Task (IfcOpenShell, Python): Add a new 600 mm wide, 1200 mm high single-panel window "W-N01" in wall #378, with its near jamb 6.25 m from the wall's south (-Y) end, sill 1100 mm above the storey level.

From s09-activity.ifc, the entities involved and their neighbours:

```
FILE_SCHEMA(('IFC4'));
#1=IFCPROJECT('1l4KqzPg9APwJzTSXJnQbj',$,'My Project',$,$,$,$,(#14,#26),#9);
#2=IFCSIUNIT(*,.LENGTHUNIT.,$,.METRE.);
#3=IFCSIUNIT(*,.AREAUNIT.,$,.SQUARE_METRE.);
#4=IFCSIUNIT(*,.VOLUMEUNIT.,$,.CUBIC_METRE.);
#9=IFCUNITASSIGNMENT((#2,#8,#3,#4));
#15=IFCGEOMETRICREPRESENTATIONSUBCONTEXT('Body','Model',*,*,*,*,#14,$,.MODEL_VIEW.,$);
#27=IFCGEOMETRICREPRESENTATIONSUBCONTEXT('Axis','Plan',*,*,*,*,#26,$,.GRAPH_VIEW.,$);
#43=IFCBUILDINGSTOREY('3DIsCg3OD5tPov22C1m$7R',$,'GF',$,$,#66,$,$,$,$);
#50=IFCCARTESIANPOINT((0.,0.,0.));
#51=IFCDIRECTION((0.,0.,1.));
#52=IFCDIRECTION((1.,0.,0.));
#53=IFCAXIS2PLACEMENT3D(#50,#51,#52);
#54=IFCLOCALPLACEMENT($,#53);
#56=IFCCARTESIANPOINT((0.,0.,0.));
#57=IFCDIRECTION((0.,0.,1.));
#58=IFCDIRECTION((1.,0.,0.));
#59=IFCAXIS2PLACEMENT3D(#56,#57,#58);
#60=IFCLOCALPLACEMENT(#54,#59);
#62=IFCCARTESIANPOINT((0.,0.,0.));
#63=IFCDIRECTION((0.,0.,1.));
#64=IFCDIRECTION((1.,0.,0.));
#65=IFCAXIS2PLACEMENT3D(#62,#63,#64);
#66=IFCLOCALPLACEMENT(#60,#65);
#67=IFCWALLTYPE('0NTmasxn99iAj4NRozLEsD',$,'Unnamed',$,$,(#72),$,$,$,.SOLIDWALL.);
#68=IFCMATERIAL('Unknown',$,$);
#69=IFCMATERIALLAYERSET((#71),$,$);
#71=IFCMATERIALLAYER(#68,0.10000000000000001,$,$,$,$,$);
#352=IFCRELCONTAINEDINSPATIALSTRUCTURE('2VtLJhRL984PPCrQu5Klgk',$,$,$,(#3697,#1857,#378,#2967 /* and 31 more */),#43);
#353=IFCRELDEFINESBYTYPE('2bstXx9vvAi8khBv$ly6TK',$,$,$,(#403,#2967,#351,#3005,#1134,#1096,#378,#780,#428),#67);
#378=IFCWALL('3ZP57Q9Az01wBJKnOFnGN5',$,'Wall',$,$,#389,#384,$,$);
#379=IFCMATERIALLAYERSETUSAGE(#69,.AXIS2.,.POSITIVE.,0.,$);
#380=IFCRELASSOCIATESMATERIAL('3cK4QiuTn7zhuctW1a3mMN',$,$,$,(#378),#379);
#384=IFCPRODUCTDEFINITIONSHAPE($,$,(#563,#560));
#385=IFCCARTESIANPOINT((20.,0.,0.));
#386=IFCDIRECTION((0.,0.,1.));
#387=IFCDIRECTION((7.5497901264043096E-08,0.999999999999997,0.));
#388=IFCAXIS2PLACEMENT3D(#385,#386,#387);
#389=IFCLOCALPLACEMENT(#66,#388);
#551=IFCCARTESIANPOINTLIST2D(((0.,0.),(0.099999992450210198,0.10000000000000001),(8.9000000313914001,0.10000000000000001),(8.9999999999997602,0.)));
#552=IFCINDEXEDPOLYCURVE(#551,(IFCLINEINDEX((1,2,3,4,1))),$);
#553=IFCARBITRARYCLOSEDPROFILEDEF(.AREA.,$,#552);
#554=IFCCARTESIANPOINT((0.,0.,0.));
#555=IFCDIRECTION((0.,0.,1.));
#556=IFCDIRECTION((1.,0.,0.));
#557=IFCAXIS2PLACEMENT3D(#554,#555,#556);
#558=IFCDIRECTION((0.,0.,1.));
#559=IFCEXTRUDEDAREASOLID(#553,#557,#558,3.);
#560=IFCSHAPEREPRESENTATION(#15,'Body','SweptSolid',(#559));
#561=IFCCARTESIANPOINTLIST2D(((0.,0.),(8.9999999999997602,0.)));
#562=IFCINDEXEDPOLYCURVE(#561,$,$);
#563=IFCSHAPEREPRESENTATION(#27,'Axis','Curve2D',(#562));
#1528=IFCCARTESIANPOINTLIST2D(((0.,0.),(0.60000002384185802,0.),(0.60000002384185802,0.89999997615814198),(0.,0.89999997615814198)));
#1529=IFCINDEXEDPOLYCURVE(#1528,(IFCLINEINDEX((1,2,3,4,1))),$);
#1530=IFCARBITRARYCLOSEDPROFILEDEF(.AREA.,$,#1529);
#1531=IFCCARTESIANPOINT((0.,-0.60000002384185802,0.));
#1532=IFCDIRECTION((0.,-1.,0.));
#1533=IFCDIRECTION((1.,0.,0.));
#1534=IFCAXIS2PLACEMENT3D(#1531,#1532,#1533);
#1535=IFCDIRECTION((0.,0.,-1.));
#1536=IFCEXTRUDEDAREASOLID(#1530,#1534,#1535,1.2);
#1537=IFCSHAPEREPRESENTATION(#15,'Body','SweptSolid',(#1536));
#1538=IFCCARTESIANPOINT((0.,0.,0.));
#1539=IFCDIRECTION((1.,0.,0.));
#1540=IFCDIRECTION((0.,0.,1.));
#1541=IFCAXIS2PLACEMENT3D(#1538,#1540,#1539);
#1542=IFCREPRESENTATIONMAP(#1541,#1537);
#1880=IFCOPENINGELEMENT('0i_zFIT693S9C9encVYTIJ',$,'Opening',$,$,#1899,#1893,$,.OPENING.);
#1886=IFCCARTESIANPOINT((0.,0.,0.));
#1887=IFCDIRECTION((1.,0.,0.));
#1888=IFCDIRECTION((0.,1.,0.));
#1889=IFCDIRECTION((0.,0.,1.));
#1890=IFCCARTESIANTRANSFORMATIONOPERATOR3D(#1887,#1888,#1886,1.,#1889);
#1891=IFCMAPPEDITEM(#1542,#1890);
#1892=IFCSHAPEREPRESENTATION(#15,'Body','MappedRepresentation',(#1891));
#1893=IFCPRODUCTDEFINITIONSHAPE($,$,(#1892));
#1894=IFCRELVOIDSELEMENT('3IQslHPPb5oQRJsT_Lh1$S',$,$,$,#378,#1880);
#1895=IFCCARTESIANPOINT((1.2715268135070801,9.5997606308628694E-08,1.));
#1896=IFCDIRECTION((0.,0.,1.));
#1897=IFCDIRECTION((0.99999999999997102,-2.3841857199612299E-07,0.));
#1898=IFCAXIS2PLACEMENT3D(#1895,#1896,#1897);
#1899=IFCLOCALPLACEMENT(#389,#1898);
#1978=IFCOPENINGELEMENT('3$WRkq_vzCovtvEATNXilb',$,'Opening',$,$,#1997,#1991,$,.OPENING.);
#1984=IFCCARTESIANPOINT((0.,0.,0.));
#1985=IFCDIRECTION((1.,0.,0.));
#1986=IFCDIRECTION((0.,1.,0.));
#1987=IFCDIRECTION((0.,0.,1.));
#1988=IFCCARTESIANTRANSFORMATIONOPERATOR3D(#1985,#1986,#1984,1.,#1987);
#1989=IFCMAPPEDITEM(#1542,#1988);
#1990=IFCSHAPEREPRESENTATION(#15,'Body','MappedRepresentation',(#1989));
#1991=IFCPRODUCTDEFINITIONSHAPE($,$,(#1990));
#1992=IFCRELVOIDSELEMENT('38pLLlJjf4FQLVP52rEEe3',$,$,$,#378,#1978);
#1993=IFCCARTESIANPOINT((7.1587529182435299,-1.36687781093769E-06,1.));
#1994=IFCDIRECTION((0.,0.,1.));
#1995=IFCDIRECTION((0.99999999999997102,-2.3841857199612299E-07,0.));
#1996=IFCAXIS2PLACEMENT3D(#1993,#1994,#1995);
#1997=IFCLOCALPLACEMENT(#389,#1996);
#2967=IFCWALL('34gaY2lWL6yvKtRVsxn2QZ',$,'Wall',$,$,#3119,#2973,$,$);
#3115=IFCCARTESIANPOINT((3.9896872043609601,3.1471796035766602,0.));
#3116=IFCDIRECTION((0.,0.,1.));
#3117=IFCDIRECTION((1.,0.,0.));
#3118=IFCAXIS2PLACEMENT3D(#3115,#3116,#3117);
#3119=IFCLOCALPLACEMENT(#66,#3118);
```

```python
import numpy as np
import ifcopenshell
import ifcopenshell.api.feature
import ifcopenshell.api.geometry
import ifcopenshell.api.root
import ifcopenshell.api.spatial
import ifcopenshell.geom
import ifcopenshell.util.element
import ifcopenshell.util.placement
import ifcopenshell.util.representation
import ifcopenshell.util.shape
import ifcopenshell.util.unit

model = ifcopenshell.open("s09-activity.ifc")
unit_scale = ifcopenshell.util.unit.calculate_unit_scale(model)
settings = ifcopenshell.geom.settings()


def volume(element):
    """Net volume in cubic metres, openings subtracted."""
    shape = ifcopenshell.geom.create_shape(settings, element)
    return ifcopenshell.util.shape.get_volume(shape.geometry)


wall = model.by_id(378)
storey = ifcopenshell.util.element.get_container(wall, ifc_class="IfcBuildingStorey")
context = ifcopenshell.util.representation.get_context(model, "Model", "Body", "MODEL_VIEW")
before = volume(wall)

width, height, from_end, sill = 0.6, 1.2, 6.25, 1.1  # metres

# The wall runs along its own X axis, and the end named is its -X end.
wall_shape = ifcopenshell.geom.create_shape(settings, wall)
x, y, z = ifcopenshell.util.shape.get_vertices(wall_shape.geometry).T
start = x.min() + from_end
face, thickness = float(y.min()), float(y.max() - y.min())
wall_matrix = ifcopenshell.util.placement.get_local_placement(wall.ObjectPlacement)
level = ifcopenshell.util.placement.get_local_placement(storey.ObjectPlacement)[2, 3]


def in_wall(x, y):
    """Placement at x, y metres in the wall's axes, at sill height."""
    matrix = wall_matrix.copy()
    matrix[:, 3] = wall_matrix @ np.array([x / unit_scale, y / unit_scale, 0.0, 1.0])
    matrix[2, 3] = level + sill / unit_scale
    return matrix


# Opening: a box that overshoots both wall faces by 50 mm.
opening = ifcopenshell.api.root.create_entity(model, ifc_class="IfcOpeningElement", predefined_type="OPENING")
box = ifcopenshell.api.geometry.add_wall_representation(
    model, context=context, length=width, height=height, thickness=thickness + 0.1
)
ifcopenshell.api.geometry.assign_representation(model, product=opening, representation=box)
ifcopenshell.api.geometry.edit_object_placement(model, product=opening, matrix=in_wall(start, face - 0.05), is_si=False)
ifcopenshell.api.feature.add_feature(model, feature=opening, element=wall)

window = ifcopenshell.api.root.create_entity(model, ifc_class="IfcWindow", name="W-N01", predefined_type="WINDOW")
window.OverallWidth, window.OverallHeight = width / unit_scale, height / unit_scale
window.PartitioningType = "SINGLE_PANEL"
body = ifcopenshell.api.geometry.add_window_representation(
    model,
    context=context,
    overall_width=window.OverallWidth,
    overall_height=window.OverallHeight,
    partition_type="SINGLE_PANEL",
)
ifcopenshell.api.geometry.assign_representation(model, product=window, representation=body)
ifcopenshell.api.spatial.assign_container(model, products=[window], relating_structure=storey)
ifcopenshell.api.feature.add_filling(model, opening=opening, element=window)

# Centre the window in the wall's thickness.
ifcopenshell.api.geometry.edit_object_placement(model, product=window, matrix=in_wall(start, face), is_si=False)
window_shape = ifcopenshell.geom.create_shape(settings, window)
depth = ifcopenshell.util.shape.get_vertices(window_shape.geometry)[:, 1]
offset = face + thickness / 2 - (depth.min() + depth.max()) / 2
ifcopenshell.api.geometry.edit_object_placement(model, product=window, matrix=in_wall(start, offset), is_si=False)

after = volume(wall)

print(f"wall volume {before:.3f} -> {after:.3f} m3")

model.write("s09-activity_v2.ifc")
```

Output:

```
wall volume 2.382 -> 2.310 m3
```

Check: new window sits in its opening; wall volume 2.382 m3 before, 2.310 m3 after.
